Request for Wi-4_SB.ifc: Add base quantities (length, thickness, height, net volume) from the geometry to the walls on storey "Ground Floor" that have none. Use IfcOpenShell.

First a look at what the model holds.

```python
import ifcopenshell
import ifcopenshell.util.element
import ifcopenshell.util.unit

model = ifcopenshell.open("Wi-4_SB.ifc")
print(model.schema)
for unit_type in ("LENGTHUNIT", "AREAUNIT", "VOLUMEUNIT"):
    print(unit_type, ifcopenshell.util.unit.calculate_unit_scale(model, unit_type))
storey = next(s for s in model.by_type("IfcBuildingStorey") if s.Name == "Ground Floor")
walls = [e for e in ifcopenshell.util.element.get_decomposition(storey) if e.is_a("IfcWall")]
for e in sorted(walls, key=lambda e: e.id()):
    print(e.id(), e.is_a(), e.Name, list(ifcopenshell.util.element.get_psets(e, qtos_only=True)), sep=" | ")
```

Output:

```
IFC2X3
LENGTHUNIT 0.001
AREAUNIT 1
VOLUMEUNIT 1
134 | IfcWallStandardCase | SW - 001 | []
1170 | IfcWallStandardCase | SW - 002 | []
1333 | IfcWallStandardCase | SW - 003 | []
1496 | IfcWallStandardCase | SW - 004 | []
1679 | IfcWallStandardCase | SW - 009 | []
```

```python
import ifcopenshell
import ifcopenshell.api.pset
import ifcopenshell.geom
import ifcopenshell.util.element
import ifcopenshell.util.shape
import ifcopenshell.util.unit

model = ifcopenshell.open("Wi-4_SB.ifc")
unit_scale = ifcopenshell.util.unit.calculate_unit_scale(model)
volume_scale = ifcopenshell.util.unit.calculate_unit_scale(model, "VOLUMEUNIT")
settings = ifcopenshell.geom.settings()

storey = next(s for s in model.by_type("IfcBuildingStorey") if s.Name == "Ground Floor")
walls = [e for e in ifcopenshell.util.element.get_decomposition(storey) if e.is_a("IfcWall")]

for e in sorted(walls, key=lambda e: e.id()):
    if ifcopenshell.util.element.get_psets(e, qtos_only=True, should_inherit=False):
        continue
    # Geometry comes back in metres, in the element's own axes.
    shape = ifcopenshell.geom.create_shape(settings, e)
    values = {
        "Length": ifcopenshell.util.shape.get_x(shape.geometry) / unit_scale,
        "Width": ifcopenshell.util.shape.get_y(shape.geometry) / unit_scale,
        "Height": ifcopenshell.util.shape.get_z(shape.geometry) / unit_scale,
        "NetVolume": ifcopenshell.util.shape.get_volume(shape.geometry) / volume_scale,
    }
    qto = ifcopenshell.api.pset.add_qto(model, product=e, name="BaseQuantities")
    ifcopenshell.api.pset.edit_qto(model, qto=qto, properties=values)
    print(e.id(), {k: round(v, 3) for k, v in values.items()})

model.write("Wi-4_SB_updated.ifc")
```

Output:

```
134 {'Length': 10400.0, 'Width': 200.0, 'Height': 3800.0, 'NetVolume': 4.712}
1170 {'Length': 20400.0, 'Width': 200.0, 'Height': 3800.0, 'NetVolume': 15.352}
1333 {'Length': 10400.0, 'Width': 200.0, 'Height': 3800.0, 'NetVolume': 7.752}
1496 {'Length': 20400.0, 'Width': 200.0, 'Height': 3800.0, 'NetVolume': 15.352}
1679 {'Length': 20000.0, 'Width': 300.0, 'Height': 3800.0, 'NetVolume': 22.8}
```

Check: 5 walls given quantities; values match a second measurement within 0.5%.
